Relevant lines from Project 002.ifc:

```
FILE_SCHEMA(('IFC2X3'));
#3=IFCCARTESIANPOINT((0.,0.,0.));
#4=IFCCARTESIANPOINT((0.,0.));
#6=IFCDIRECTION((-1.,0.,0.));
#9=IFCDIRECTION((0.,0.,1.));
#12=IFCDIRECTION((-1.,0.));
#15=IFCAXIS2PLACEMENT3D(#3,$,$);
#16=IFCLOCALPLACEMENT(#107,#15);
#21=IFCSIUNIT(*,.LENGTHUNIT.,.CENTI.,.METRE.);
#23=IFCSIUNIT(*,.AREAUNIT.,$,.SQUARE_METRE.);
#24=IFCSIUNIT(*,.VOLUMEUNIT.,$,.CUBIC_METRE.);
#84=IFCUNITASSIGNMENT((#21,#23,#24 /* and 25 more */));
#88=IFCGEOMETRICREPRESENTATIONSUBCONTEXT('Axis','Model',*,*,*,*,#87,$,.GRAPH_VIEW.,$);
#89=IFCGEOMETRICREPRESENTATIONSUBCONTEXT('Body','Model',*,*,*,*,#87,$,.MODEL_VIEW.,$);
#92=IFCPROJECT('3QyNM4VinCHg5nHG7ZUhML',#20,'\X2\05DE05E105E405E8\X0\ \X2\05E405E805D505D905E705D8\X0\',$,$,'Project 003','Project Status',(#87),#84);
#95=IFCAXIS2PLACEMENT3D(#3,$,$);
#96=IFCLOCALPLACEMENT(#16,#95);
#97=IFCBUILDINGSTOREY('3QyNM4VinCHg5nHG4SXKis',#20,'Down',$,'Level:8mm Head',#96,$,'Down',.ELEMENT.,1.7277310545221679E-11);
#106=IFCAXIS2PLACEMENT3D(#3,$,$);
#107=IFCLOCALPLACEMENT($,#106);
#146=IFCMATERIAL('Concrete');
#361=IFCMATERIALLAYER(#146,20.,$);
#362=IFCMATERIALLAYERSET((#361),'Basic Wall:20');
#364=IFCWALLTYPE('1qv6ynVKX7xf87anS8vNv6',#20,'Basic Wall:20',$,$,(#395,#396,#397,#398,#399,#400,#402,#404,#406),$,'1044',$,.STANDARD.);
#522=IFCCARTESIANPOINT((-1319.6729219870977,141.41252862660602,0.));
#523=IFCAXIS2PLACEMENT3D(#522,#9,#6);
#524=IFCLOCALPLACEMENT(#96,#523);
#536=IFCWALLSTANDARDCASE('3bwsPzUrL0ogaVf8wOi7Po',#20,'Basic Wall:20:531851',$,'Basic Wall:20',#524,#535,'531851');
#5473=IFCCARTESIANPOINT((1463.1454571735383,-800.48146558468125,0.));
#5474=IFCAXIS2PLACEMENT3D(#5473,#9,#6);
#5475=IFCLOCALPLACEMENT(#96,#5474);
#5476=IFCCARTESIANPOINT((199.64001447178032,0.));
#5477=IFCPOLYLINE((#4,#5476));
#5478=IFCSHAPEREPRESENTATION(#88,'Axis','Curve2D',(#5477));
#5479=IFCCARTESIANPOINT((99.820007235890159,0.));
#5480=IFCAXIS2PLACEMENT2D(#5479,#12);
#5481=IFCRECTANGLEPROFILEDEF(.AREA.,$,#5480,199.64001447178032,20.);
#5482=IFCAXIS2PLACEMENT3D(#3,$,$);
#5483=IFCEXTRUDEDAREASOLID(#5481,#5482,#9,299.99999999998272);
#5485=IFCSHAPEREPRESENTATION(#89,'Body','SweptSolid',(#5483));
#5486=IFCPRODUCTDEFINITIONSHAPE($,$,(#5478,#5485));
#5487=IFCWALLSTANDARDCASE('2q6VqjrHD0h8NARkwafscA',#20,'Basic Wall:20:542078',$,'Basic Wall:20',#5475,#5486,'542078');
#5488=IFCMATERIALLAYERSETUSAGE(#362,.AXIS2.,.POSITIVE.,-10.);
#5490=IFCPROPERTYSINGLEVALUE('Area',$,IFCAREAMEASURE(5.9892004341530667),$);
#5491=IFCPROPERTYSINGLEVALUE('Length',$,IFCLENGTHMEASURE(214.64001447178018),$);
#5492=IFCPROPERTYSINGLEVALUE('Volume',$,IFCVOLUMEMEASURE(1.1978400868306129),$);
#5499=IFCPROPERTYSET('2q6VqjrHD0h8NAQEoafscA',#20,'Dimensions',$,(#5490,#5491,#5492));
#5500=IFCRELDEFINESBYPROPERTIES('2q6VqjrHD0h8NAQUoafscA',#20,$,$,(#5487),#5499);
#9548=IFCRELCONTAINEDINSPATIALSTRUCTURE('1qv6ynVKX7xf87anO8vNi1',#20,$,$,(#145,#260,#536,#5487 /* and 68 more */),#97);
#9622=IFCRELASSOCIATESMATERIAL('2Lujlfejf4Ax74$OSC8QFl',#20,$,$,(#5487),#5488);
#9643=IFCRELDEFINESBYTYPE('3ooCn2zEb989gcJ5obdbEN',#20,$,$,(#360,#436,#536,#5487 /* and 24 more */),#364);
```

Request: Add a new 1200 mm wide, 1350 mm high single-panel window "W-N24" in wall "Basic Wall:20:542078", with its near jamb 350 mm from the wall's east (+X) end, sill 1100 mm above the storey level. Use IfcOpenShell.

```python
import numpy as np
import ifcopenshell
import ifcopenshell.api.feature
import ifcopenshell.api.geometry
import ifcopenshell.api.pset
import ifcopenshell.api.root
import ifcopenshell.api.spatial
import ifcopenshell.api.type
import ifcopenshell.geom
import ifcopenshell.util.element
import ifcopenshell.util.placement
import ifcopenshell.util.representation
import ifcopenshell.util.shape
import ifcopenshell.util.unit

model = ifcopenshell.open("Project 002.ifc")
unit_scale = ifcopenshell.util.unit.calculate_unit_scale(model)
area_scale = ifcopenshell.util.unit.calculate_unit_scale(model, "AREAUNIT")
volume_scale = ifcopenshell.util.unit.calculate_unit_scale(model, "VOLUMEUNIT")
settings = ifcopenshell.geom.settings()


def volume(element):
    """Net volume in cubic metres, openings subtracted."""
    shape = ifcopenshell.geom.create_shape(settings, element)
    return ifcopenshell.util.shape.get_volume(shape.geometry)


wall = model.by_guid("2q6VqjrHD0h8NARkwafscA")
storey = ifcopenshell.util.element.get_container(wall, ifc_class="IfcBuildingStorey")
context = ifcopenshell.util.representation.get_context(model, "Model", "Body", "MODEL_VIEW")
before = volume(wall)

width, height, from_end, sill = 1.2, 1.35, 0.35, 1.1  # metres

# The wall runs along its own X axis, and the end named is its -X end.
wall_shape = ifcopenshell.geom.create_shape(settings, wall)
x, y, z = ifcopenshell.util.shape.get_vertices(wall_shape.geometry).T
start = x.min() + from_end
face, thickness = float(y.min()), float(y.max() - y.min())
wall_matrix = ifcopenshell.util.placement.get_local_placement(wall.ObjectPlacement)
level = ifcopenshell.util.placement.get_local_placement(storey.ObjectPlacement)[2, 3]


def in_wall(x, y):
    """Placement at x, y metres in the wall's axes, at sill height."""
    matrix = wall_matrix.copy()
    matrix[:, 3] = wall_matrix @ np.array([x / unit_scale, y / unit_scale, 0.0, 1.0])
    matrix[2, 3] = level + sill / unit_scale
    return matrix


# Opening: a box that overshoots both wall faces by 50 mm.
opening = ifcopenshell.api.root.create_entity(model, ifc_class="IfcOpeningElement")
box = ifcopenshell.api.geometry.add_wall_representation(
    model, context=context, length=width, height=height, thickness=thickness + 0.1
)
ifcopenshell.api.geometry.assign_representation(model, product=opening, representation=box)
ifcopenshell.api.geometry.edit_object_placement(model, product=opening, matrix=in_wall(start, face - 0.05), is_si=False)
ifcopenshell.api.feature.add_feature(model, feature=opening, element=wall)

window = ifcopenshell.api.root.create_entity(model, ifc_class="IfcWindow", name="W-N24")
window.OverallWidth, window.OverallHeight = width / unit_scale, height / unit_scale
body = ifcopenshell.api.geometry.add_window_representation(
    model,
    context=context,
    overall_width=window.OverallWidth,
    overall_height=window.OverallHeight,
    partition_type="SINGLE_PANEL",
)
ifcopenshell.api.geometry.assign_representation(model, product=window, representation=body)
ifcopenshell.api.spatial.assign_container(model, products=[window], relating_structure=storey)
fills = ifcopenshell.api.feature.add_filling(model, opening=opening, element=window)
fills.OwnerHistory = window.OwnerHistory  # required in IFC2X3

# IFC2X3 keeps the operation on the window style.
style = ifcopenshell.api.root.create_entity(model, ifc_class="IfcWindowStyle", name="W-N24")
style.OperationType, style.ConstructionType = "SINGLE_PANEL", "NOTDEFINED"
style.ParameterTakesPrecedence = style.Sizeable = False
ifcopenshell.api.type.assign_type(model, related_objects=[window], relating_type=style)

# Centre the window in the wall's thickness.
ifcopenshell.api.geometry.edit_object_placement(model, product=window, matrix=in_wall(start, face), is_si=False)
window_shape = ifcopenshell.geom.create_shape(settings, window)
depth = ifcopenshell.util.shape.get_vertices(window_shape.geometry)[:, 1]
offset = face + thickness / 2 - (depth.min() + depth.max()) / 2
ifcopenshell.api.geometry.edit_object_placement(model, product=window, matrix=in_wall(start, offset), is_si=False)

after = volume(wall)

# Update the wall's stored quantities.
pset = model.by_id(ifcopenshell.util.element.get_pset(wall, "Dimensions", should_inherit=False)["id"])
ifcopenshell.api.pset.edit_pset(model, pset=pset, properties={
    "Area": model.create_entity("IfcAreaMeasure", after / thickness / area_scale),
    "Volume": model.create_entity("IfcVolumeMeasure", after / volume_scale),
})

print(f"wall volume {before:.3f} -> {after:.3f} m3")

model.write("Project 002_rev.ifc")
```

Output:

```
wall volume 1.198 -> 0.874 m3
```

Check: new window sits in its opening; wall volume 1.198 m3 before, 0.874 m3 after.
